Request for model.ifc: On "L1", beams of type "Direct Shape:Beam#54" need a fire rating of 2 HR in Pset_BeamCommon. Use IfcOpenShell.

First a look at what the model holds.

```python
import ifcopenshell
import ifcopenshell.util.element

model = ifcopenshell.open("model.ifc")
print(model.schema)
storey = next(s for s in model.by_type("IfcBuildingStorey") if s.Name == "L1")
beams = [e for e in ifcopenshell.util.element.get_decomposition(storey) if e.is_a("IfcBeam")]
seen = {}
for e in beams:
    element_type = ifcopenshell.util.element.get_type(e)
    key = (element_type.Name if element_type != e and element_type else None, ifcopenshell.util.element.get_pset(e, "Pset_BeamCommon", "FireRating"))
    seen[key] = seen.get(key, 0) + 1
for (name, value), count in sorted(seen.items(), key=str):
    print(count, "x", name, "|", value)
```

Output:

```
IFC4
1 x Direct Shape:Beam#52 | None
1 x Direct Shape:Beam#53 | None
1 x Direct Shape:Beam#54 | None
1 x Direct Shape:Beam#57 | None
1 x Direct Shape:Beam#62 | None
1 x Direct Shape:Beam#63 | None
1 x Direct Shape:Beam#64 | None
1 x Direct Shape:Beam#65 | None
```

```python
import ifcopenshell
import ifcopenshell.api.pset
import ifcopenshell.util.element

model = ifcopenshell.open("model.ifc")

storey = next(s for s in model.by_type("IfcBuildingStorey") if s.Name == "L1")
beams = [e for e in ifcopenshell.util.element.get_decomposition(storey) if e.is_a("IfcBeam")]

count = 0
for e in beams:
    element_type = ifcopenshell.util.element.get_type(e)
    if element_type in (None, e) or element_type.Name != "Direct Shape:Beam#54":
        continue
    # add_pset returns the element's existing set when there is one.
    pset = ifcopenshell.api.pset.add_pset(model, product=e, name="Pset_BeamCommon")
    ifcopenshell.api.pset.edit_pset(model, pset=pset, properties={"FireRating": "2 HR"})
    count += 1

print(count, "beams updated")

model.write("model-out.ifc")
```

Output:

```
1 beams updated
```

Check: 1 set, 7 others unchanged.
